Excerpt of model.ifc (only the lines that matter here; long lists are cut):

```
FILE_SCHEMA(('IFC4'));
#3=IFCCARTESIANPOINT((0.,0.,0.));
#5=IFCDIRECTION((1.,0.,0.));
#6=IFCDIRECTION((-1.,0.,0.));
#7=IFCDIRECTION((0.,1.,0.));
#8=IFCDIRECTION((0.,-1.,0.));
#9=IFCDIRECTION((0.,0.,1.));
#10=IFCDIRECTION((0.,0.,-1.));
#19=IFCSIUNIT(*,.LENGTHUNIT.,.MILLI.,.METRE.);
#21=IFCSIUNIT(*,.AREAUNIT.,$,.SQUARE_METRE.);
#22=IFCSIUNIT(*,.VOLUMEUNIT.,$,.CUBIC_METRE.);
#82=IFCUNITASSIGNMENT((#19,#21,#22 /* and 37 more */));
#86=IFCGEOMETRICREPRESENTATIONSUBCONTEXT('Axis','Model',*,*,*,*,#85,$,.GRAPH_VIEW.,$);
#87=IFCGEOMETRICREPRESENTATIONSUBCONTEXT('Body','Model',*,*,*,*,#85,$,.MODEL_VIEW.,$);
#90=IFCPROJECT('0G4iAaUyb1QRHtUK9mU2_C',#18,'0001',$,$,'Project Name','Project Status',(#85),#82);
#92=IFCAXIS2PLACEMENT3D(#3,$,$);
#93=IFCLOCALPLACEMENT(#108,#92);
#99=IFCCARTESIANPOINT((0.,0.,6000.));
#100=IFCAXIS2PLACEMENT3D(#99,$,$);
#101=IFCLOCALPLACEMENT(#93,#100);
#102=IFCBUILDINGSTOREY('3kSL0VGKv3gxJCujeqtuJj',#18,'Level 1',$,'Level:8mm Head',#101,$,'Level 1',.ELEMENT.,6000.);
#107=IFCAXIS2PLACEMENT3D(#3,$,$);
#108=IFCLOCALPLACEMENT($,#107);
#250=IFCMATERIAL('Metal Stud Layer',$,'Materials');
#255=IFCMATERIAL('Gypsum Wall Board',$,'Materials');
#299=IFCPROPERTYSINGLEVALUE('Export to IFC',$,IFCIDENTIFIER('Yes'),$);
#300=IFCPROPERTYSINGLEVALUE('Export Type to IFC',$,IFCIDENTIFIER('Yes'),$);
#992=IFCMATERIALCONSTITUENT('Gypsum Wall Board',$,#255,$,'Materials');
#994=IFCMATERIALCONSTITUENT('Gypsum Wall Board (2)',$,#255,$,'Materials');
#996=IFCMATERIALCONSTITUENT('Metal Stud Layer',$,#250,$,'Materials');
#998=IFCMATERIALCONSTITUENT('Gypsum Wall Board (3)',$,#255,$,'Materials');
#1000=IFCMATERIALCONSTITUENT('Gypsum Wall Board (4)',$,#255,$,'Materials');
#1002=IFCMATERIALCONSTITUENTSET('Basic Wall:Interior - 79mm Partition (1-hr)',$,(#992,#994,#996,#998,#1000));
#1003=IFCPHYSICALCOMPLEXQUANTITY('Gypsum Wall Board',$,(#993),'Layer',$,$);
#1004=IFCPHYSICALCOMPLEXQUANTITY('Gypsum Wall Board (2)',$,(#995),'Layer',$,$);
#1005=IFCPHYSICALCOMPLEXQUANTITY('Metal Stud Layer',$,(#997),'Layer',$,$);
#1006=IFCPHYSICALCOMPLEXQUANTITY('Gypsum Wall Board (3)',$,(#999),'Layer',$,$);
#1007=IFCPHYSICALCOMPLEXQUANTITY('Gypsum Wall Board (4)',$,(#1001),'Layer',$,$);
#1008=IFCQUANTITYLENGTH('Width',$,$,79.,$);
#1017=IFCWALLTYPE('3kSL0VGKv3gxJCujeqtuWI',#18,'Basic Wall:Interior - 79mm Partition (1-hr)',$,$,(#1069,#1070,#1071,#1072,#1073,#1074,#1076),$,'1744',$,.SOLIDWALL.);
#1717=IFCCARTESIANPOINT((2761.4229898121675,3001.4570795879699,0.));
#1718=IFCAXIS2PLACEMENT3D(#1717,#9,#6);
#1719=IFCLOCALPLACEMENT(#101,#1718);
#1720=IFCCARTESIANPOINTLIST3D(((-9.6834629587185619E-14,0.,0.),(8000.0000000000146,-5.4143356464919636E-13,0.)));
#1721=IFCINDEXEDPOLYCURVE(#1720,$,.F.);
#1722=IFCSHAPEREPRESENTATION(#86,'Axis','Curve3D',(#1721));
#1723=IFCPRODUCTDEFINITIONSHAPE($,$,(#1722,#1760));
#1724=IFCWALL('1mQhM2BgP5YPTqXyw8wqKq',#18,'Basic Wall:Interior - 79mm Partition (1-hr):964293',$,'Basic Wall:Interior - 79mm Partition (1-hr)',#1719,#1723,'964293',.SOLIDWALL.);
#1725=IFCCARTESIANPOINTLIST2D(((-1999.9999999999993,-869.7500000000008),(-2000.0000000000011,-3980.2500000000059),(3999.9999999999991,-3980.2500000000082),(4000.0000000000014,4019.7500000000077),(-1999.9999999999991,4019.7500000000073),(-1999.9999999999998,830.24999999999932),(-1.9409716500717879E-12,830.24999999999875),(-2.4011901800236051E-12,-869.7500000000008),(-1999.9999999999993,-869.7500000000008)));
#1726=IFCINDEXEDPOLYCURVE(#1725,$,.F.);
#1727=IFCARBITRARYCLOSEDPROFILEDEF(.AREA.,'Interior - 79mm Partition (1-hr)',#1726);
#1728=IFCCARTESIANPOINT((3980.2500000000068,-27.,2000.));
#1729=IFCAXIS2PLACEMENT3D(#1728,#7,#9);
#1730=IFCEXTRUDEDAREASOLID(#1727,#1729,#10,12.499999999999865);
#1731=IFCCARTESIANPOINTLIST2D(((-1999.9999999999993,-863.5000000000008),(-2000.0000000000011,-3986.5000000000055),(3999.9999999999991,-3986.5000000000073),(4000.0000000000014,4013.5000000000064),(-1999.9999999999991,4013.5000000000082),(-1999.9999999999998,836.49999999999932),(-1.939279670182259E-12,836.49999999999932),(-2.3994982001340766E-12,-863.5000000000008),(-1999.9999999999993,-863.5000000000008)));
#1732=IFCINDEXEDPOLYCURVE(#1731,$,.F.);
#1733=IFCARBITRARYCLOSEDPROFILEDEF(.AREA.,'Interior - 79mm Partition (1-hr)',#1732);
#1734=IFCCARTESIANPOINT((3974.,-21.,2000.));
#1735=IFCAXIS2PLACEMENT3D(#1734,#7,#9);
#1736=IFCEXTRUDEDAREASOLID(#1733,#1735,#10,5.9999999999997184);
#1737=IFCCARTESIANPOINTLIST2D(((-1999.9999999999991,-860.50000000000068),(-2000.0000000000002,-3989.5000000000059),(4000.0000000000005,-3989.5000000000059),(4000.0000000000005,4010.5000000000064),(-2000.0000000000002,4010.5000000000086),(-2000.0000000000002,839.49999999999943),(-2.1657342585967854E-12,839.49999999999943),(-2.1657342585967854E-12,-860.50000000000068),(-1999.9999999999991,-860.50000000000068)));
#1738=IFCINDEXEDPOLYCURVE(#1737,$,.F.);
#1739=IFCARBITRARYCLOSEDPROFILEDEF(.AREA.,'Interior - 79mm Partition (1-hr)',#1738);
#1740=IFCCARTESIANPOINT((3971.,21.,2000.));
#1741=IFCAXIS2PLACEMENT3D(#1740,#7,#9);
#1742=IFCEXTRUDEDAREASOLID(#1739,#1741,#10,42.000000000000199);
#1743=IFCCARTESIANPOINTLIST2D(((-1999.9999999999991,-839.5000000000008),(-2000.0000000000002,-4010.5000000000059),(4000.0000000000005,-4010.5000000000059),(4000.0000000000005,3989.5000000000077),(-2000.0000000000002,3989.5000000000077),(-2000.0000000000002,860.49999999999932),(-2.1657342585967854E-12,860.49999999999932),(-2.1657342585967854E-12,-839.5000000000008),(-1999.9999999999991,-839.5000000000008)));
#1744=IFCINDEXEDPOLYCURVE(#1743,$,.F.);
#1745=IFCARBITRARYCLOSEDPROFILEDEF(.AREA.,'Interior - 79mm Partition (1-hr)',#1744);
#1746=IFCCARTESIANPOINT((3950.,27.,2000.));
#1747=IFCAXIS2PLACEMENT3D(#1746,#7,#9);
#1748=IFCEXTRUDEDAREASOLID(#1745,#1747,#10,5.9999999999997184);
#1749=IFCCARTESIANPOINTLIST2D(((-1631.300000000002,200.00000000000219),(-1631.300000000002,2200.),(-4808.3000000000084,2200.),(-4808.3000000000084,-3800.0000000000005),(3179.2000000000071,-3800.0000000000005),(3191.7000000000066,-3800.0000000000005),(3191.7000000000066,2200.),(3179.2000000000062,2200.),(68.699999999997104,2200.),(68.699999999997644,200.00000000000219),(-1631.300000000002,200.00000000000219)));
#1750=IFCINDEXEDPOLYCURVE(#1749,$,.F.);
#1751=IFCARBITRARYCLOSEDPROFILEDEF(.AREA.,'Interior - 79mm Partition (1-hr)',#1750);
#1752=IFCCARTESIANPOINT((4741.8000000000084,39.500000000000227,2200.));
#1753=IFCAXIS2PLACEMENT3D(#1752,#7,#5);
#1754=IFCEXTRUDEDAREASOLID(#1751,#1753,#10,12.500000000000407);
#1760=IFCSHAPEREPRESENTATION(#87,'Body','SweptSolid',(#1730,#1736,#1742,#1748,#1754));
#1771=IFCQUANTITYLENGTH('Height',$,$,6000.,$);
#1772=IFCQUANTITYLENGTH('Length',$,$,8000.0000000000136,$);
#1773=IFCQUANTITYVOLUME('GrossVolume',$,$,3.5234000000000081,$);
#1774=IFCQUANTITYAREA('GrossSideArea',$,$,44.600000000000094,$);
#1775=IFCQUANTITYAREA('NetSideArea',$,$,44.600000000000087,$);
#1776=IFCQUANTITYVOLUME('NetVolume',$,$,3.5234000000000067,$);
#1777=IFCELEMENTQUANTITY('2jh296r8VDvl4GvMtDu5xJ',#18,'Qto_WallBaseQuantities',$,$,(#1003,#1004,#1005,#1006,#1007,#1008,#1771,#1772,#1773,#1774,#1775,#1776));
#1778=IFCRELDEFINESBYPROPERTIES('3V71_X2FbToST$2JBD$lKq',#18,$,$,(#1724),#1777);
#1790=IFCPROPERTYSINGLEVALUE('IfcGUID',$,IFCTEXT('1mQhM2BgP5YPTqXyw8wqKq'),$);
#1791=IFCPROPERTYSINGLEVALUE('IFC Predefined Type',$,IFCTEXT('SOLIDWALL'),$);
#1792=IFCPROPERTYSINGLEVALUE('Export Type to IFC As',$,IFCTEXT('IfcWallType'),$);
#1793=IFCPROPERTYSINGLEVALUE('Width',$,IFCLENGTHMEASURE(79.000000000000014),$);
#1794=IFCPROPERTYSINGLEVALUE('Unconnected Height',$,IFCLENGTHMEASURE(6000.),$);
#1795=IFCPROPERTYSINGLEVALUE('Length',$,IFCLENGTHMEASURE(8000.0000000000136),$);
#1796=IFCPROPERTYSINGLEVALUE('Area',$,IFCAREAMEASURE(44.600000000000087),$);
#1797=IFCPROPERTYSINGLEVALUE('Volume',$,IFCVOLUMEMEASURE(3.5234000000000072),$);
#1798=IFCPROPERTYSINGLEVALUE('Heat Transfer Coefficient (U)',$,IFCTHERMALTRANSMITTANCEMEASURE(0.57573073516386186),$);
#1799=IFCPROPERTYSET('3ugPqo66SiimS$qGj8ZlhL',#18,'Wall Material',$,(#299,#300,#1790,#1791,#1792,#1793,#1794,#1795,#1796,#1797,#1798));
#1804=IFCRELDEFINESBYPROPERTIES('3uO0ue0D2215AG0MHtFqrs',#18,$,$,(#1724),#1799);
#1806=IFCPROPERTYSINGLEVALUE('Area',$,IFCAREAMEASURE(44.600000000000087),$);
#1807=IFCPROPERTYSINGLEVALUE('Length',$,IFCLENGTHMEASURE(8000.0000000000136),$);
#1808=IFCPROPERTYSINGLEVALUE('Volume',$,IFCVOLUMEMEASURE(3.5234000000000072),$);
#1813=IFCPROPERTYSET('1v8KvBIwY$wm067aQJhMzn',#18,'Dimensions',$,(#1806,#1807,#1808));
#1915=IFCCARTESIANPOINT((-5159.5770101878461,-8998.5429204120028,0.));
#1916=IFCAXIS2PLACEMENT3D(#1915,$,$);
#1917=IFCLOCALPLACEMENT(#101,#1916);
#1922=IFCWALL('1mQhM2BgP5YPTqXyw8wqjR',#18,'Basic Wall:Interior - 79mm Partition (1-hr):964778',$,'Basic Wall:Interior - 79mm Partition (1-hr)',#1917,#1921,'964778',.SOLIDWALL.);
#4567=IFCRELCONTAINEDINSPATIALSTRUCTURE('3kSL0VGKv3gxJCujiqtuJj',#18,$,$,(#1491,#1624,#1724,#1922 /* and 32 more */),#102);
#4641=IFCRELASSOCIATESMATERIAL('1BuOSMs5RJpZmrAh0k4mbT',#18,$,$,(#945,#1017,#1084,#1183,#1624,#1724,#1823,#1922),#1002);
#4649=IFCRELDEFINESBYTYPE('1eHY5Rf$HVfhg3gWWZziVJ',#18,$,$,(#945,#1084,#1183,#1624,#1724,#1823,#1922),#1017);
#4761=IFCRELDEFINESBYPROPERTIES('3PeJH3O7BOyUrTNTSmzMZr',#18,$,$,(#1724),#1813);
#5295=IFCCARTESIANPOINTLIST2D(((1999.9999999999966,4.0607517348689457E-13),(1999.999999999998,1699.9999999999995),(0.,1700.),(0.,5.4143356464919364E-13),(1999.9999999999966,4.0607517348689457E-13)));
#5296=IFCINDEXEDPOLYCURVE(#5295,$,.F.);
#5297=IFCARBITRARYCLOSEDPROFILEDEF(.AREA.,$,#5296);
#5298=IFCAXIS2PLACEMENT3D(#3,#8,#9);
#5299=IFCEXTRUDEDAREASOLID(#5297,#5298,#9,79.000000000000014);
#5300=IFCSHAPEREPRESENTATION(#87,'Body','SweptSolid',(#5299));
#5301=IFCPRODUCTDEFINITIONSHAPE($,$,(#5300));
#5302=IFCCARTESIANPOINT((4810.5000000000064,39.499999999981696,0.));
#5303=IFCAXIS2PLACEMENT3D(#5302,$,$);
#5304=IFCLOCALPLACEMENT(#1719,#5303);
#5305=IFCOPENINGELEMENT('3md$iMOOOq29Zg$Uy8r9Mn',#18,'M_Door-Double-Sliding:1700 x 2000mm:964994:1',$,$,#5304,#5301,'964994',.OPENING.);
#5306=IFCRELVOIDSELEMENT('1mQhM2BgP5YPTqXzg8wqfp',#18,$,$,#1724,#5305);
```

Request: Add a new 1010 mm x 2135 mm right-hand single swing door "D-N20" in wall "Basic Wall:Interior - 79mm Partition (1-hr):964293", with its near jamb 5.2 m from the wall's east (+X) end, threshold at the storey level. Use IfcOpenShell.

```python
import numpy as np
import ifcopenshell
import ifcopenshell.api.feature
import ifcopenshell.api.geometry
import ifcopenshell.api.pset
import ifcopenshell.api.root
import ifcopenshell.api.spatial
import ifcopenshell.geom
import ifcopenshell.util.element
import ifcopenshell.util.placement
import ifcopenshell.util.representation
import ifcopenshell.util.shape
import ifcopenshell.util.unit

model = ifcopenshell.open("model.ifc")
unit_scale = ifcopenshell.util.unit.calculate_unit_scale(model)
area_scale = ifcopenshell.util.unit.calculate_unit_scale(model, "AREAUNIT")
volume_scale = ifcopenshell.util.unit.calculate_unit_scale(model, "VOLUMEUNIT")
settings = ifcopenshell.geom.settings()


def volume(element):
    """Net volume in cubic metres, openings subtracted."""
    shape = ifcopenshell.geom.create_shape(settings, element)
    return ifcopenshell.util.shape.get_volume(shape.geometry)


wall = model.by_guid("1mQhM2BgP5YPTqXyw8wqKq")
storey = ifcopenshell.util.element.get_container(wall, ifc_class="IfcBuildingStorey")
context = ifcopenshell.util.representation.get_context(model, "Model", "Body", "MODEL_VIEW")
before = volume(wall)

width, height, from_end, sill = 1.01, 2.135, 5.2, 0.0  # metres

# The wall runs along its own X axis, and the end named is its -X end.
wall_shape = ifcopenshell.geom.create_shape(settings, wall)
x, y, z = ifcopenshell.util.shape.get_vertices(wall_shape.geometry).T
start = x.min() + from_end
face, thickness = float(y.min()), float(y.max() - y.min())
wall_matrix = ifcopenshell.util.placement.get_local_placement(wall.ObjectPlacement)
level = ifcopenshell.util.placement.get_local_placement(storey.ObjectPlacement)[2, 3]


def in_wall(x, y):
    """Placement at x, y metres in the wall's axes, at sill height."""
    matrix = wall_matrix.copy()
    matrix[:, 3] = wall_matrix @ np.array([x / unit_scale, y / unit_scale, 0.0, 1.0])
    matrix[2, 3] = level + sill / unit_scale
    return matrix


# Opening: a box that overshoots both wall faces by 50 mm.
opening = ifcopenshell.api.root.create_entity(model, ifc_class="IfcOpeningElement", predefined_type="OPENING")
box = ifcopenshell.api.geometry.add_wall_representation(
    model, context=context, length=width, height=height, thickness=thickness + 0.1
)
ifcopenshell.api.geometry.assign_representation(model, product=opening, representation=box)
ifcopenshell.api.geometry.edit_object_placement(model, product=opening, matrix=in_wall(start, face - 0.05), is_si=False)
ifcopenshell.api.feature.add_feature(model, feature=opening, element=wall)

door = ifcopenshell.api.root.create_entity(model, ifc_class="IfcDoor", name="D-N20", predefined_type="DOOR")
door.OverallWidth, door.OverallHeight = width / unit_scale, height / unit_scale
door.OperationType = "SINGLE_SWING_RIGHT"
body = ifcopenshell.api.geometry.add_door_representation(
    model,
    context=context,
    overall_width=door.OverallWidth,
    overall_height=door.OverallHeight,
    operation_type="SINGLE_SWING_RIGHT",
    lining_properties={"LiningDepth": thickness / unit_scale, "ThresholdDepth": thickness / unit_scale},
)
ifcopenshell.api.geometry.assign_representation(model, product=door, representation=body)
ifcopenshell.api.spatial.assign_container(model, products=[door], relating_structure=storey)
ifcopenshell.api.feature.add_filling(model, opening=opening, element=door)

# The lining spans the wall, so the door starts at the wall face.
ifcopenshell.api.geometry.edit_object_placement(model, product=door, matrix=in_wall(start, face), is_si=False)

after = volume(wall)

# Update the wall's stored quantities.
qto = model.by_id(ifcopenshell.util.element.get_pset(wall, "Qto_WallBaseQuantities", should_inherit=False)["id"])
ifcopenshell.api.pset.edit_qto(model, qto=qto, properties={
    "NetSideArea": after / thickness / area_scale,
    "NetVolume": after / volume_scale,
})
pset = model.by_id(ifcopenshell.util.element.get_pset(wall, "Wall Material", should_inherit=False)["id"])
ifcopenshell.api.pset.edit_pset(model, pset=pset, properties={
    "Area": model.create_entity("IfcAreaMeasure", after / thickness / area_scale),
    "Volume": model.create_entity("IfcVolumeMeasure", after / volume_scale),
})
pset = model.by_id(ifcopenshell.util.element.get_pset(wall, "Dimensions", should_inherit=False)["id"])
ifcopenshell.api.pset.edit_pset(model, pset=pset, properties={
    "Area": model.create_entity("IfcAreaMeasure", after / thickness / area_scale),
    "Volume": model.create_entity("IfcVolumeMeasure", after / volume_scale),
})

print(f"wall volume {before:.3f} -> {after:.3f} m3")

model.write("model_rev.ifc")
```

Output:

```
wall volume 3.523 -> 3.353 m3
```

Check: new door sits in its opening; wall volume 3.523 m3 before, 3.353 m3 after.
